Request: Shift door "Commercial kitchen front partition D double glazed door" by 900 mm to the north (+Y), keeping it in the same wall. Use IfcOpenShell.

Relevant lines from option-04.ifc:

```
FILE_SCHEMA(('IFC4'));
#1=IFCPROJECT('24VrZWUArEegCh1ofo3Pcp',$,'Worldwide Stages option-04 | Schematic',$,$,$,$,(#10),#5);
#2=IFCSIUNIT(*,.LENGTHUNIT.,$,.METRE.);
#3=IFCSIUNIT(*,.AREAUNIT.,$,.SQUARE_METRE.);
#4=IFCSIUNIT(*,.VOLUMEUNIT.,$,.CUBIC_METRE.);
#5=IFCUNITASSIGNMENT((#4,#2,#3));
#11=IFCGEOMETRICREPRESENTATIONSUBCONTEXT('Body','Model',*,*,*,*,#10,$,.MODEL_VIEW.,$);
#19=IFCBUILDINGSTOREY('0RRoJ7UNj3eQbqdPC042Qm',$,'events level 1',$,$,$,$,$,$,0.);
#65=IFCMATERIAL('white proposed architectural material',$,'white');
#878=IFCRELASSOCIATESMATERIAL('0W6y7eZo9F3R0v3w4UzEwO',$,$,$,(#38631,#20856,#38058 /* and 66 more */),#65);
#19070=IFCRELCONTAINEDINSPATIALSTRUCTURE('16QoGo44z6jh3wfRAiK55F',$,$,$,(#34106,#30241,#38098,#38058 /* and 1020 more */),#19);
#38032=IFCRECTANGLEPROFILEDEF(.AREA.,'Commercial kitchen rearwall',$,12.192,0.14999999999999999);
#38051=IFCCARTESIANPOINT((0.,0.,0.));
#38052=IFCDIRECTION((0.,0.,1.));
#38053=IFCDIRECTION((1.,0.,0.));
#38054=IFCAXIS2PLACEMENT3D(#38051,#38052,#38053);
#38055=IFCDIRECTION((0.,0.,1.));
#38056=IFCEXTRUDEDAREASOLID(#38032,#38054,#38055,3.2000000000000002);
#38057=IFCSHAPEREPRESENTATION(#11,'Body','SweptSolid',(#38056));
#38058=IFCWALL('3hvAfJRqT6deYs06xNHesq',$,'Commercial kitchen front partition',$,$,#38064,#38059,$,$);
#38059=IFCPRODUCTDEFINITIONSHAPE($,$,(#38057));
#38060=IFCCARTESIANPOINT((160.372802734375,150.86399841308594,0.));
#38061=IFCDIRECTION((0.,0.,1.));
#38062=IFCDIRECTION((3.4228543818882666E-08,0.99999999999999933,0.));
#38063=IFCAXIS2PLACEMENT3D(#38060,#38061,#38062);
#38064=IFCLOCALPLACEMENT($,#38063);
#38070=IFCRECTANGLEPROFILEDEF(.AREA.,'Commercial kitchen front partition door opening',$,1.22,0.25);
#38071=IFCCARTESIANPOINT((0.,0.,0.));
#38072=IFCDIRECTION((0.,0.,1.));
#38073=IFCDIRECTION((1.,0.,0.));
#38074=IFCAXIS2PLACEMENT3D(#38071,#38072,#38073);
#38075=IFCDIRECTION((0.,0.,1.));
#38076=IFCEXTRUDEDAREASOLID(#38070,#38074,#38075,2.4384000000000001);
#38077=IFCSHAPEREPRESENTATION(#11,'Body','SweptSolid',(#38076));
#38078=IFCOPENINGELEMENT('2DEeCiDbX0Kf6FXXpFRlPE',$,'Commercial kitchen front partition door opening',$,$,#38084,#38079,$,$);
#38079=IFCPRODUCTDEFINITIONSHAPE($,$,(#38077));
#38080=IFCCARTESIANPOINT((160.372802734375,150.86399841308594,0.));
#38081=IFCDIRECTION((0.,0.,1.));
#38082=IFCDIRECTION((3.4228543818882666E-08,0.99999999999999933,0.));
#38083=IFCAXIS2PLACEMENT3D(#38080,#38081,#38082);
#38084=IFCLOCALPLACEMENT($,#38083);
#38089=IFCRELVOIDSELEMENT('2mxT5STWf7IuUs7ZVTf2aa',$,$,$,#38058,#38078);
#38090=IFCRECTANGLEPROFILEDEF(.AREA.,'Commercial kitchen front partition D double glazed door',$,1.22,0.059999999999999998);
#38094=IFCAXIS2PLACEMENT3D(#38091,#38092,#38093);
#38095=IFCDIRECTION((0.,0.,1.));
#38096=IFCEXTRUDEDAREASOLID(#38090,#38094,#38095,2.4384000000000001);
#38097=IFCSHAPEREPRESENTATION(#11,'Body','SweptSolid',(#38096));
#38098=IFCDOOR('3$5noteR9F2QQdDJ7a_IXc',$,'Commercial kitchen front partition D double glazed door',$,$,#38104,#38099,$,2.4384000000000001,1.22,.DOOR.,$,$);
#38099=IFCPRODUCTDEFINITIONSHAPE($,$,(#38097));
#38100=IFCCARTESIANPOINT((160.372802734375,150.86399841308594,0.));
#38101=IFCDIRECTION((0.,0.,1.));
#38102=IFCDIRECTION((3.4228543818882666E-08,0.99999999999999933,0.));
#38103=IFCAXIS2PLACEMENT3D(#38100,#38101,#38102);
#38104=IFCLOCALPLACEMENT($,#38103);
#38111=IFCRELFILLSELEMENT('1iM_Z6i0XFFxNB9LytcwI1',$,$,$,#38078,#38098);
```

```python
import ifcopenshell
import ifcopenshell.api.geometry
import ifcopenshell.util.placement

model = ifcopenshell.open("option-04.ifc")

door = model.by_guid("3$5noteR9F2QQdDJ7a_IXc")
opening = door.FillsVoids[0].RelatingOpeningElement
wall = opening.VoidsElements[0].RelatingBuildingElement

wall_matrix = ifcopenshell.util.placement.get_local_placement(wall.ObjectPlacement)
shift = wall_matrix[:3, 0] * 0.9
before = ifcopenshell.util.placement.get_local_placement(door.ObjectPlacement)[:3, 3].copy()

# The door is not placed relative to its opening, so move both.
for product in (opening, door):
    matrix = ifcopenshell.util.placement.get_local_placement(product.ObjectPlacement)
    matrix[:3, 3] += shift
    ifcopenshell.api.geometry.edit_object_placement(model, product=product, matrix=matrix, is_si=False)

after = ifcopenshell.util.placement.get_local_placement(door.ObjectPlacement)[:3, 3]
print("door moved by", (after - before).round(3) + 0.0)

model.write("option-04_v2.ifc")
```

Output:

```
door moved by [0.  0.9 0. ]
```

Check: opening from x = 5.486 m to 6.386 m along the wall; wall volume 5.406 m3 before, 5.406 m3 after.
